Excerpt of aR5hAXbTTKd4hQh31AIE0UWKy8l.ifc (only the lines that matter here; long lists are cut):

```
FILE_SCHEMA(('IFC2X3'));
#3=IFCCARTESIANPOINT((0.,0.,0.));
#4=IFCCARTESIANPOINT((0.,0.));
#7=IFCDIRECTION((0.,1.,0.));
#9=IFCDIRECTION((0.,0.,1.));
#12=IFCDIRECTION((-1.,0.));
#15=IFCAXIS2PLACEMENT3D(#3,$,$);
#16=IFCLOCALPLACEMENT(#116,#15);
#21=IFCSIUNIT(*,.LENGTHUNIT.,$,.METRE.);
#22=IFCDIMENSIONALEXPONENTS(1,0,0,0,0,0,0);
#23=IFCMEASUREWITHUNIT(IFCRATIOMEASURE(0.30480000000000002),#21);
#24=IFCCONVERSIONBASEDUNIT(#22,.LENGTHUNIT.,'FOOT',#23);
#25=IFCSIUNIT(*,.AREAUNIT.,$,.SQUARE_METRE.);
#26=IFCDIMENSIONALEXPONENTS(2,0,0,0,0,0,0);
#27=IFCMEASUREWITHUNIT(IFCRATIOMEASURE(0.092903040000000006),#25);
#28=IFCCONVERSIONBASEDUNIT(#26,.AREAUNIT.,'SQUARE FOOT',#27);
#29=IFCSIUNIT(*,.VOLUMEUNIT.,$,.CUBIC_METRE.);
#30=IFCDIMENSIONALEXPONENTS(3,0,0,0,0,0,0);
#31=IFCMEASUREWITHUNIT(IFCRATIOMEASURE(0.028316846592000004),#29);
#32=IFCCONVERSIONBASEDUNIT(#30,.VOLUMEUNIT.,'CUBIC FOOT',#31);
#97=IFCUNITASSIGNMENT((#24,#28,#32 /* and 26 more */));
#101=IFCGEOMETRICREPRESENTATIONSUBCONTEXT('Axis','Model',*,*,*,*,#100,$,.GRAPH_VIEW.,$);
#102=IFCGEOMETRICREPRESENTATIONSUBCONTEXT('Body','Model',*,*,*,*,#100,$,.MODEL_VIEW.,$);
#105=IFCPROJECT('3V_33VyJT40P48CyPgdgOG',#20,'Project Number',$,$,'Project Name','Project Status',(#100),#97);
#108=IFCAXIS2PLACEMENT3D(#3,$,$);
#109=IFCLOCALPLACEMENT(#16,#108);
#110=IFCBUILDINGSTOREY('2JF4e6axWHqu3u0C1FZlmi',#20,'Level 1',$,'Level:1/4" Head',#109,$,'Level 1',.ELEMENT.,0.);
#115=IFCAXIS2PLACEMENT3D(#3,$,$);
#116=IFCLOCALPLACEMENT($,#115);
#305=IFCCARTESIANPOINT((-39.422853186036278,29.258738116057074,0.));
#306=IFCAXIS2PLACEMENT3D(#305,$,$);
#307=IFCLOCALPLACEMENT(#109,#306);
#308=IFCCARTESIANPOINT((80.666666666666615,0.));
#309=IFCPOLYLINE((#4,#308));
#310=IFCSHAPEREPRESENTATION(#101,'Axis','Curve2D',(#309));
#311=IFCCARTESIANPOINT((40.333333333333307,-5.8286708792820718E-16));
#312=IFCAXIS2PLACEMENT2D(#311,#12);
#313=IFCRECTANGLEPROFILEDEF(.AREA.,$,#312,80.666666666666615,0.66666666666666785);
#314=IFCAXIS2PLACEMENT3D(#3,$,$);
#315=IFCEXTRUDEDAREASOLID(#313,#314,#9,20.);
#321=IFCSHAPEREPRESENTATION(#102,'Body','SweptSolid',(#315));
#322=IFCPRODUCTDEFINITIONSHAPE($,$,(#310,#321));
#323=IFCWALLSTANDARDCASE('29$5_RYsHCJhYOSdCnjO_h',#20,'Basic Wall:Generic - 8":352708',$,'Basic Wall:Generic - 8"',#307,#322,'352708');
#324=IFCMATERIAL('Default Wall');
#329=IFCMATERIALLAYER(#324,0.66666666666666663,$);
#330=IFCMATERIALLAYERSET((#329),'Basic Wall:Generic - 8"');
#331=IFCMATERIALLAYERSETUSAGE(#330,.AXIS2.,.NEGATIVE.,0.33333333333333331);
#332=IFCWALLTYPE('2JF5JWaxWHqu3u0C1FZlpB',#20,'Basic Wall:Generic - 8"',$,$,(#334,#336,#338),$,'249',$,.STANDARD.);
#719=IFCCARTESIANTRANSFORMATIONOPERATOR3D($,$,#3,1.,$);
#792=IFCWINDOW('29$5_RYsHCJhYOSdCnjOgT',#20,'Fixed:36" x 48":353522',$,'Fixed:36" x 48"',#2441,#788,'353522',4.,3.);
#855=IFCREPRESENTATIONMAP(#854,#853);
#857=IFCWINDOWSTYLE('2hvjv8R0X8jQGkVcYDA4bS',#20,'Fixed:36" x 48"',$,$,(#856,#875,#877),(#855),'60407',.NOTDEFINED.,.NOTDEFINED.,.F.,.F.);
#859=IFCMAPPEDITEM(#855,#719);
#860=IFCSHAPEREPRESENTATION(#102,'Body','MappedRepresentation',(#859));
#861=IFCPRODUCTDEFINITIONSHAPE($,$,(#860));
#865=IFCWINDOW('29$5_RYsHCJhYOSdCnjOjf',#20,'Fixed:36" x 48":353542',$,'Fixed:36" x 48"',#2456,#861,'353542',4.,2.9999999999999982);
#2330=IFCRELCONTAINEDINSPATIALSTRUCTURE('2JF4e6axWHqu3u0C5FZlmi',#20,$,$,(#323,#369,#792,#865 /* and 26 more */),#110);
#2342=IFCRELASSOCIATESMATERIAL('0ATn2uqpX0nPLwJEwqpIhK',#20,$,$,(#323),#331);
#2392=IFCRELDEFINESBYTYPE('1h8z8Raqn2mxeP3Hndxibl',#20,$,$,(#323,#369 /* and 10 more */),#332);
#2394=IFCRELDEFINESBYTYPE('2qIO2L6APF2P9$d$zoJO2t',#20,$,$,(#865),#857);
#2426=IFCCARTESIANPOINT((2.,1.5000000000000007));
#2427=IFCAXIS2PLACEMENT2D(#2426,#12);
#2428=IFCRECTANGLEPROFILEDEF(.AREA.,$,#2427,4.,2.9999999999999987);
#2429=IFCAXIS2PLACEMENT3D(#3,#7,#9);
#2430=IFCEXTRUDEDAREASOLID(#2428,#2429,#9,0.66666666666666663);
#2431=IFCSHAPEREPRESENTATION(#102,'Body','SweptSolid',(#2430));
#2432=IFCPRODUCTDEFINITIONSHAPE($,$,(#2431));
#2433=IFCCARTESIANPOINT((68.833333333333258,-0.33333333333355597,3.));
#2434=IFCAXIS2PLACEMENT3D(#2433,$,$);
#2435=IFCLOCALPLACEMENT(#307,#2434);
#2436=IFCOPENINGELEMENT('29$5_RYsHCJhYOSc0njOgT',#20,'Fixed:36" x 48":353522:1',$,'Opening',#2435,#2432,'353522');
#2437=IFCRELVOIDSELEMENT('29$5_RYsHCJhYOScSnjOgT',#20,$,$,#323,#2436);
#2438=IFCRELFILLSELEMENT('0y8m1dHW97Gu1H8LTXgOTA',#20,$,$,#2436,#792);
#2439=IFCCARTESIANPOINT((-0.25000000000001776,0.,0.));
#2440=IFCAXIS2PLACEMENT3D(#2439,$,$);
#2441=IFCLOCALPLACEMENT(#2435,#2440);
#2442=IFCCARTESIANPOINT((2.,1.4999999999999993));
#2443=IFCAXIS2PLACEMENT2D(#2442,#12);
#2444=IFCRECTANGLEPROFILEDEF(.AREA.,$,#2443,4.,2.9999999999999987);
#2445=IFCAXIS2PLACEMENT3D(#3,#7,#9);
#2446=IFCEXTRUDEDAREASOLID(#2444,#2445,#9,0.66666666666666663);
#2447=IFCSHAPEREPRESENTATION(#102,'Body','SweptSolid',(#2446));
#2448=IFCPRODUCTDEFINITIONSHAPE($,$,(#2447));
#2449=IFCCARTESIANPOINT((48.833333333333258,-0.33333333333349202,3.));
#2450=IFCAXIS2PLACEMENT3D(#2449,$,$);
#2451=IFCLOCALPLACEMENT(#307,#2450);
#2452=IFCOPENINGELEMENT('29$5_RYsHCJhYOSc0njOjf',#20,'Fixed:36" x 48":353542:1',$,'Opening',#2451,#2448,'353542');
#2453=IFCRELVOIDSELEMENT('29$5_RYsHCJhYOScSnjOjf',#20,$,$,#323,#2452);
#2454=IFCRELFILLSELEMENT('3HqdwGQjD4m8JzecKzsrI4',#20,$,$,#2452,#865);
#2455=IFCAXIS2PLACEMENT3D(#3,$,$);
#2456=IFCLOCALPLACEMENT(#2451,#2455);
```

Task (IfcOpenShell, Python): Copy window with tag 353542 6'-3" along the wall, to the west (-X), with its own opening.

```python
import ifcopenshell
import ifcopenshell.api.feature
import ifcopenshell.api.geometry
import ifcopenshell.api.root
import ifcopenshell.geom
import ifcopenshell.util.element
import ifcopenshell.util.placement
import ifcopenshell.util.shape
import ifcopenshell.util.unit

model = ifcopenshell.open("aR5hAXbTTKd4hQh31AIE0UWKy8l.ifc")
unit_scale = ifcopenshell.util.unit.calculate_unit_scale(model)
settings = ifcopenshell.geom.settings()


def volume(element):
    """Net volume in cubic metres, openings subtracted."""
    shape = ifcopenshell.geom.create_shape(settings, element)
    return ifcopenshell.util.shape.get_volume(shape.geometry)


def reuse_history(source, copy):
    """copy_class also copies each property set's owner history, people and application; keep the originals."""
    for rel in copy.IsDefinedBy:
        if rel.is_a("IfcRelDefinesByProperties") and (history := rel.RelatingPropertyDefinition.OwnerHistory):
            rel.RelatingPropertyDefinition.OwnerHistory = source.OwnerHistory
            ifcopenshell.util.element.remove_deep2(model, history)


window = model.by_guid("29$5_RYsHCJhYOSdCnjOjf")
opening = window.FillsVoids[0].RelatingOpeningElement
wall = opening.VoidsElements[0].RelatingBuildingElement
before = volume(wall)
shift = ifcopenshell.util.placement.get_local_placement(wall.ObjectPlacement)[:3, 0] * -75 * 0.0254 / unit_scale

# copy_class copies the void relationship, type, container and properties, but no geometry.
new_opening = ifcopenshell.api.root.copy_class(model, product=opening)
new_opening.Representation = ifcopenshell.util.element.copy_deep(
    model, opening.Representation, exclude=["IfcGeometricRepresentationContext", "IfcRepresentationMap"]
)
new_opening.Name = 'Fixed:36" x 48"'
new_opening.Tag = None
new_window = ifcopenshell.api.root.copy_class(model, product=window)
new_window.Representation = ifcopenshell.util.element.copy_deep(
    model, window.Representation, exclude=["IfcGeometricRepresentationContext", "IfcRepresentationMap"]
)
new_window.Name = 'Fixed:36" x 48"'
new_window.Tag = None
reuse_history(window, new_window)
fills = ifcopenshell.api.feature.add_filling(model, opening=new_opening, element=new_window)
fills.OwnerHistory = new_window.OwnerHistory  # required in IFC2X3

for old, new in ((opening, new_opening), (window, new_window)):
    matrix = ifcopenshell.util.placement.get_local_placement(old.ObjectPlacement)
    matrix[:3, 3] += shift
    ifcopenshell.api.geometry.edit_object_placement(model, product=new, matrix=matrix, is_si=False)

after = volume(wall)

print(f"wall volume {before:.3f} -> {after:.3f} m3")

model.write("aR5hAXbTTKd4hQh31AIE0UWKy8l_v2.ifc")
```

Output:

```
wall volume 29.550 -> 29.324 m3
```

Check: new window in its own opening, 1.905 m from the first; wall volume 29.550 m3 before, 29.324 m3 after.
